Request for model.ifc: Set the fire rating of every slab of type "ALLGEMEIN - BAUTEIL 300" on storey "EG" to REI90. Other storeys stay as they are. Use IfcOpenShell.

First a look at what the model holds.

```python
import ifcopenshell
import ifcopenshell.util.element

model = ifcopenshell.open("model.ifc")
print(model.schema)
storey = next(s for s in model.by_type("IfcBuildingStorey") if s.Name == "EG")
slabs = [e for e in ifcopenshell.util.element.get_decomposition(storey) if e.is_a("IfcSlab")]
seen = {}
for e in slabs:
    element_type = ifcopenshell.util.element.get_type(e)
    key = (element_type.Name if element_type != e and element_type else None, ifcopenshell.util.element.get_pset(e, "Pset_SlabCommon", "FireRating"))
    seen[key] = seen.get(key, 0) + 1
for (name, value), count in sorted(seen.items(), key=str):
    print(count, "x", name, "|", value)
```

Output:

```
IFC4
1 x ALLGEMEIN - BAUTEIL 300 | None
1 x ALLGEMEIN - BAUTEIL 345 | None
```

```python
import ifcopenshell
import ifcopenshell.api.pset
import ifcopenshell.util.element

model = ifcopenshell.open("model.ifc")

storey = next(s for s in model.by_type("IfcBuildingStorey") if s.Name == "EG")
slabs = [e for e in ifcopenshell.util.element.get_decomposition(storey) if e.is_a("IfcSlab")]

count = 0
for e in slabs:
    element_type = ifcopenshell.util.element.get_type(e)
    if element_type in (None, e) or element_type.Name != "ALLGEMEIN - BAUTEIL 300":
        continue
    # add_pset returns the element's existing set when there is one.
    pset = ifcopenshell.api.pset.add_pset(model, product=e, name="Pset_SlabCommon")
    ifcopenshell.api.pset.edit_pset(model, pset=pset, properties={"FireRating": "REI90"})
    count += 1

print(count, "slabs updated")

model.write("model_rev.ifc")
```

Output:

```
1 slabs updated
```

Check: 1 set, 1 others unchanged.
